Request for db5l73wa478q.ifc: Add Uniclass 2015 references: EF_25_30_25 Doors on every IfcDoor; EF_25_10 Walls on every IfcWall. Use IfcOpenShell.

First a look at what the model holds.

```python
import ifcopenshell

model = ifcopenshell.open("db5l73wa478q.ifc")
print(model.schema)
print("classifications:", [c.Name for c in model.by_type("IfcClassification")])
for ifc_class in ("IfcDoor", "IfcRoof", "IfcStair", "IfcWall", "IfcWindow"):
    print(ifc_class, len(model.by_type(ifc_class)))
```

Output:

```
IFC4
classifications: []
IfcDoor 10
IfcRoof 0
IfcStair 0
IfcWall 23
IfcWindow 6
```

```python
import ifcopenshell
import ifcopenshell.api.classification

model = ifcopenshell.open("db5l73wa478q.ifc")

system = ifcopenshell.api.classification.add_classification(model, classification="Uniclass 2015")

codes = {
    "IfcDoor": ("EF_25_30_25", "Doors"),
    "IfcWall": ("EF_25_10", "Walls"),
}
for ifc_class, (code, name) in codes.items():
    products = model.by_type(ifc_class)
    ifcopenshell.api.classification.add_reference(
        model, products=products, classification=system, identification=code, name=name
    )
    print(code, len(products))

model.write("db5l73wa478q_v2.ifc")
```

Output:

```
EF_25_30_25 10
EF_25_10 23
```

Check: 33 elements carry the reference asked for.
